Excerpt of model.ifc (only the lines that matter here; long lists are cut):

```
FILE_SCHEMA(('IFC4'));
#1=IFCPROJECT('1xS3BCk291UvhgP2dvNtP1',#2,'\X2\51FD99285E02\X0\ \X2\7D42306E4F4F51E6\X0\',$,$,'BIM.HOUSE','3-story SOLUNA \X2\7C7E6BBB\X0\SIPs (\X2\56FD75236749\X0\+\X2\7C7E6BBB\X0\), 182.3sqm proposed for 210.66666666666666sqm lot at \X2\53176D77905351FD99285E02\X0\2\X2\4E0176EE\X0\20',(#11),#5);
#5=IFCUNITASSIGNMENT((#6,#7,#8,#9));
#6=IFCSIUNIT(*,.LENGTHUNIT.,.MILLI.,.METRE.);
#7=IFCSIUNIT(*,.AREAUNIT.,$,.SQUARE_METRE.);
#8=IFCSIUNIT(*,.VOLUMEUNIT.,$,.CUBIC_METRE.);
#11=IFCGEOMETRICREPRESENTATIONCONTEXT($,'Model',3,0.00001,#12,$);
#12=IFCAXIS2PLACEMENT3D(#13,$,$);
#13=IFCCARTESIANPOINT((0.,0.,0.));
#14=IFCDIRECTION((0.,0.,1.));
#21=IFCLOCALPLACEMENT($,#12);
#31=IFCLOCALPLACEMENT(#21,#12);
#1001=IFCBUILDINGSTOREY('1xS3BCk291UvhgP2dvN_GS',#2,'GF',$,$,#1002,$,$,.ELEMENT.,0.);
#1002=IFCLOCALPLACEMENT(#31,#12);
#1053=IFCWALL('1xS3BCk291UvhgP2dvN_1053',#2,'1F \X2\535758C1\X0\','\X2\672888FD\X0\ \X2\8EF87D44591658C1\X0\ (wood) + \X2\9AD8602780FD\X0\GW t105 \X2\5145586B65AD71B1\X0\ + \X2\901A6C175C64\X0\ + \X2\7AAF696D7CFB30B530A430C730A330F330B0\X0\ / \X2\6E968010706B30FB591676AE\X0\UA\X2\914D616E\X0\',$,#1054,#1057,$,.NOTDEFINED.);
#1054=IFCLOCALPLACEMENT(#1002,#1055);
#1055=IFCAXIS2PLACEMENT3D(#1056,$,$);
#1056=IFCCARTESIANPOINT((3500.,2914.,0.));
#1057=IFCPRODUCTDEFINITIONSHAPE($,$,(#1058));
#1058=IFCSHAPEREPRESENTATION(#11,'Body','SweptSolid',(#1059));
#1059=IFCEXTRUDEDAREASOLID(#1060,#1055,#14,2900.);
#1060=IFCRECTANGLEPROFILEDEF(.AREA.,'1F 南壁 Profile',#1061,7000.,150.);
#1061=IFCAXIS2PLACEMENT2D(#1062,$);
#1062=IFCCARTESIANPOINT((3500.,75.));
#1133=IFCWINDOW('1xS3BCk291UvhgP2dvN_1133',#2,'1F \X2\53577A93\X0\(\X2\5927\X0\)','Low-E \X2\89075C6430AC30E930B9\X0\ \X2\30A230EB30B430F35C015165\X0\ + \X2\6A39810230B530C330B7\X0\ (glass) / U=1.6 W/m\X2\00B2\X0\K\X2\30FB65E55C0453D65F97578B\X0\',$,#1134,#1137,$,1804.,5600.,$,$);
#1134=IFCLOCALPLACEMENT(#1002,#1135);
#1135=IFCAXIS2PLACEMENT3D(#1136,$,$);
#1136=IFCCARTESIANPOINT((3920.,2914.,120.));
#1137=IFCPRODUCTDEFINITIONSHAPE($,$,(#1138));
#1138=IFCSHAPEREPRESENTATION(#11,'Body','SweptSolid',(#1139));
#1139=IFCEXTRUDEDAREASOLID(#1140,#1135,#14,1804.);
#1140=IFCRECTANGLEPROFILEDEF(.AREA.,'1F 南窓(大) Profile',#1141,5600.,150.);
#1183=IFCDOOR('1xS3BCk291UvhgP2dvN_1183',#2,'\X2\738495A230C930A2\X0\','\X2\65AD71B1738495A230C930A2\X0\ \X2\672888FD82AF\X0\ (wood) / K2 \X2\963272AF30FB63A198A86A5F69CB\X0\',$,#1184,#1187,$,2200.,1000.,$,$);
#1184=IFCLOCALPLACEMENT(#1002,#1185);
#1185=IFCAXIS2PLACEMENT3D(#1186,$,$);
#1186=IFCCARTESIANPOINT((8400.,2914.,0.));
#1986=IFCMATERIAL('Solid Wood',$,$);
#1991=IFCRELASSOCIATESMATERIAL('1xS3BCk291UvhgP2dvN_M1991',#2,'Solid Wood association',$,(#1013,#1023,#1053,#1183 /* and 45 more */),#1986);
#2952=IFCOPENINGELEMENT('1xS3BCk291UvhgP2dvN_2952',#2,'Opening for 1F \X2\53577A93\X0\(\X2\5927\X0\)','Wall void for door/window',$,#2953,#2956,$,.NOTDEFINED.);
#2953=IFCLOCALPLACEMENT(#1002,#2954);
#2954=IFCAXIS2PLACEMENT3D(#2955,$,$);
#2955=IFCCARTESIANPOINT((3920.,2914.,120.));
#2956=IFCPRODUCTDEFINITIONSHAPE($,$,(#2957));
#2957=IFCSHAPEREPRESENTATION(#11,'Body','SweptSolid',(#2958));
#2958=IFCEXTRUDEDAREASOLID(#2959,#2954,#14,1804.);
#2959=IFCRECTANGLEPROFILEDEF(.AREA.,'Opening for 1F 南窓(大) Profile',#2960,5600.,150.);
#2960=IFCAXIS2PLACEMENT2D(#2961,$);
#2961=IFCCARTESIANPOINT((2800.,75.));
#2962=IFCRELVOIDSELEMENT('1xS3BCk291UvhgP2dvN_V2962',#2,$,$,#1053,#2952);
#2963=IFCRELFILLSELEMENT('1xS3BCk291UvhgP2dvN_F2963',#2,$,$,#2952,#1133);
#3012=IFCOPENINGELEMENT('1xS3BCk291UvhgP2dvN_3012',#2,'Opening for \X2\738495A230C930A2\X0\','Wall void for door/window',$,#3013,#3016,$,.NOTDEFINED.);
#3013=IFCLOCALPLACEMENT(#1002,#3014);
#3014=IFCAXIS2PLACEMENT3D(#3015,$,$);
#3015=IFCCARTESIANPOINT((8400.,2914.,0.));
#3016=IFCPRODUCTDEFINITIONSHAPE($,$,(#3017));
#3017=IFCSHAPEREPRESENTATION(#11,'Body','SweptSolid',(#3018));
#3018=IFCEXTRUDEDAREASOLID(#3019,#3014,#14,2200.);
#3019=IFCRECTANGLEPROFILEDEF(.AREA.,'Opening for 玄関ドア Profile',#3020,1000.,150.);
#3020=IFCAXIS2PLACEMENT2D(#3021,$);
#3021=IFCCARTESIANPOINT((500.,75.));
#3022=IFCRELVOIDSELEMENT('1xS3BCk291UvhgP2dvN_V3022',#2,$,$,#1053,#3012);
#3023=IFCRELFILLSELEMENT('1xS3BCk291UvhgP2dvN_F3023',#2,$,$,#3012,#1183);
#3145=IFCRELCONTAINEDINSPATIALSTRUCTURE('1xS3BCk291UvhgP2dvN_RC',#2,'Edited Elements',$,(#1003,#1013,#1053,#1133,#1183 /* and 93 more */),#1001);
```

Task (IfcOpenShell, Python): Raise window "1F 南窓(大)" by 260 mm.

```python
import numpy as np
import ifcopenshell
import ifcopenshell.api.geometry
import ifcopenshell.util.placement
import ifcopenshell.util.unit

model = ifcopenshell.open("model.ifc")
unit_scale = ifcopenshell.util.unit.calculate_unit_scale(model)

window = model.by_guid("1xS3BCk291UvhgP2dvN_1133")
opening = window.FillsVoids[0].RelatingOpeningElement
dz = 0.26 / unit_scale

shift = np.array([0.0, 0.0, dz])
# The window is not placed relative to its opening, so move both.
for product in (opening, window):
    matrix = ifcopenshell.util.placement.get_local_placement(product.ObjectPlacement)
    matrix[:3, 3] += shift
    ifcopenshell.api.geometry.edit_object_placement(model, product=product, matrix=matrix, is_si=False)

print(f"moved by {dz * unit_scale:+.3f} m")

model.write("model_v2.ifc")
```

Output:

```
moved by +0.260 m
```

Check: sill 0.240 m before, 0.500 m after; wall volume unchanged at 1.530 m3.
